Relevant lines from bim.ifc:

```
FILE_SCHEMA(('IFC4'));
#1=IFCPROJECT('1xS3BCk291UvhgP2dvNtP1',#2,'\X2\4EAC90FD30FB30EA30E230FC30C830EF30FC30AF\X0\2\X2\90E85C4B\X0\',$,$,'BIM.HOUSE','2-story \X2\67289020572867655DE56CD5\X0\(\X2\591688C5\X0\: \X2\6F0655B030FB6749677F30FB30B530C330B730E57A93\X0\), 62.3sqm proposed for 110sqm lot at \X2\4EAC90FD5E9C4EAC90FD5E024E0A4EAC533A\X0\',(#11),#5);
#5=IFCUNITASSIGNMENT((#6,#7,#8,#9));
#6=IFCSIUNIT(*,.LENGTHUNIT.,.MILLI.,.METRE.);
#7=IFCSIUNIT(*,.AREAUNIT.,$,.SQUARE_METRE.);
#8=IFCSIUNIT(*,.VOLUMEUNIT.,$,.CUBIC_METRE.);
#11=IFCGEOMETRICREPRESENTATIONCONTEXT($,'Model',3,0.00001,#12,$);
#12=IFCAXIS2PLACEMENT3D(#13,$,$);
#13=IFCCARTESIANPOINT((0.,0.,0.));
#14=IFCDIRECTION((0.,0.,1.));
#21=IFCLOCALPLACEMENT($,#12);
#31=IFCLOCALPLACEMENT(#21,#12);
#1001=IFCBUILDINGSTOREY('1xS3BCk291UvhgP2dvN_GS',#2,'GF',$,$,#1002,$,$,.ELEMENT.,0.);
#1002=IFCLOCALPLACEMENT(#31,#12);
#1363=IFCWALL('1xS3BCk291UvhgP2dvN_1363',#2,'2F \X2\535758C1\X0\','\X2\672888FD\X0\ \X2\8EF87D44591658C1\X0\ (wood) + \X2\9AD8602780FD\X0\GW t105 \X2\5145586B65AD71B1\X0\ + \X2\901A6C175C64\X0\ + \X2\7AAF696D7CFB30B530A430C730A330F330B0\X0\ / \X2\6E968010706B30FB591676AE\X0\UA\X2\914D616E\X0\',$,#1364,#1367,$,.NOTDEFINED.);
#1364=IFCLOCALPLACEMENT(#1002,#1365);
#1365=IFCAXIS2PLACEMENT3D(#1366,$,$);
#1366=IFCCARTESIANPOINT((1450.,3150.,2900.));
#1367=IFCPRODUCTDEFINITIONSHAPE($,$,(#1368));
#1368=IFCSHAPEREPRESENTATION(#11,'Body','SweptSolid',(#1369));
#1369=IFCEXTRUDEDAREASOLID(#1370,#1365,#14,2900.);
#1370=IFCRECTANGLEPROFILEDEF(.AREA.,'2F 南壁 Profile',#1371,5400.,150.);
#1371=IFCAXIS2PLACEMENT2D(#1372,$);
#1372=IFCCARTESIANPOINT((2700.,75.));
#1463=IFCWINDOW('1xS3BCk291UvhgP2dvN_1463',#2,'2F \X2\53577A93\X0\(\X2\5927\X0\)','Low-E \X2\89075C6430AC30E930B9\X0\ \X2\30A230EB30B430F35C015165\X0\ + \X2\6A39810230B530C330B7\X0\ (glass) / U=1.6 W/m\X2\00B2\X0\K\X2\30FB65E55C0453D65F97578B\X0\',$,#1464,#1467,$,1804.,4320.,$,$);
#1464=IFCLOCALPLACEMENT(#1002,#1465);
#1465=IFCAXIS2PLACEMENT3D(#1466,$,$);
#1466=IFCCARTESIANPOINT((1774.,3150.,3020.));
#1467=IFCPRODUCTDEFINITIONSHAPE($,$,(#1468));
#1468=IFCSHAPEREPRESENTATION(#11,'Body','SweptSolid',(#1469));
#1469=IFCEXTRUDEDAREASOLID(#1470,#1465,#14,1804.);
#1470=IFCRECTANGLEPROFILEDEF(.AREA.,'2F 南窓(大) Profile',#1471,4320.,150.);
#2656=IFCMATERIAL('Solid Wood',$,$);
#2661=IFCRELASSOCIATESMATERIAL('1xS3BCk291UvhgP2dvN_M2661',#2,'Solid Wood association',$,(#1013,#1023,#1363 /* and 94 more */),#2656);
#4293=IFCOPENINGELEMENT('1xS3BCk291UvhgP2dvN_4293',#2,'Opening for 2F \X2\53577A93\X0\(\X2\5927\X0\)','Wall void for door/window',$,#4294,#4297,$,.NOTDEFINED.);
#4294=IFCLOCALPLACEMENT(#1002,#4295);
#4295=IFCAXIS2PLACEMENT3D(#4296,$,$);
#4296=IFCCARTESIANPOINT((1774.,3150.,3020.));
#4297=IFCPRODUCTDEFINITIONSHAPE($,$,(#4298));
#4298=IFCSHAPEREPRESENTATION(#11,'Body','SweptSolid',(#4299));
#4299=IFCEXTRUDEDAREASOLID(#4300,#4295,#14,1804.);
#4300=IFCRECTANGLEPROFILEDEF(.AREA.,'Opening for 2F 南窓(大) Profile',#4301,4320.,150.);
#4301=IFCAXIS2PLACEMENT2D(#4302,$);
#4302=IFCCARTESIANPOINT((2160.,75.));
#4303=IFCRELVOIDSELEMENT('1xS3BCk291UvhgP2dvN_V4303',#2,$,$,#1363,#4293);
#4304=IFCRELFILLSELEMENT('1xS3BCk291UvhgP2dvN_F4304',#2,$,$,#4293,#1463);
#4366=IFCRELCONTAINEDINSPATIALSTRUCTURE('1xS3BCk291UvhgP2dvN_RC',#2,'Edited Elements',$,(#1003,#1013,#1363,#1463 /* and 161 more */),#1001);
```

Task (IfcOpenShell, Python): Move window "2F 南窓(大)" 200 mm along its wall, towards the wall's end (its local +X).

```python
import ifcopenshell
import ifcopenshell.api.geometry
import ifcopenshell.util.placement
import ifcopenshell.util.unit

model = ifcopenshell.open("bim.ifc")
unit_scale = ifcopenshell.util.unit.calculate_unit_scale(model)

window = model.by_id(1463)
opening = window.FillsVoids[0].RelatingOpeningElement
wall = opening.VoidsElements[0].RelatingBuildingElement

wall_matrix = ifcopenshell.util.placement.get_local_placement(wall.ObjectPlacement)
shift = wall_matrix[:3, 0] * 0.2 / unit_scale
before = ifcopenshell.util.placement.get_local_placement(window.ObjectPlacement)[:3, 3].copy()

# The window is not placed relative to its opening, so move both.
for product in (opening, window):
    matrix = ifcopenshell.util.placement.get_local_placement(product.ObjectPlacement)
    matrix[:3, 3] += shift
    ifcopenshell.api.geometry.edit_object_placement(model, product=product, matrix=matrix, is_si=False)

after = ifcopenshell.util.placement.get_local_placement(window.ObjectPlacement)[:3, 3]
print("window moved by", (after - before).round(3) + 0.0)

model.write("bim_v2.ifc")
```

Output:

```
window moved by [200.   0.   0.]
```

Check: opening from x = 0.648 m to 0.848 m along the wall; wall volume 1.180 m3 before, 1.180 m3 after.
